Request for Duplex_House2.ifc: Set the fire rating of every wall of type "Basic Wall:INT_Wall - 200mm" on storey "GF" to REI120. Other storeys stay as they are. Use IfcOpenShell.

First a look at what the model holds.

```python
import ifcopenshell
import ifcopenshell.util.element

model = ifcopenshell.open("Duplex_House2.ifc")
print(model.schema)
storey = next(s for s in model.by_type("IfcBuildingStorey") if s.Name == "GF")
walls = [e for e in ifcopenshell.util.element.get_decomposition(storey) if e.is_a("IfcWall")]
seen = {}
for e in walls:
    element_type = ifcopenshell.util.element.get_type(e)
    key = (element_type.Name if element_type != e and element_type else None, ifcopenshell.util.element.get_pset(e, "Pset_WallCommon", "FireRating"))
    seen[key] = seen.get(key, 0) + 1
for (name, value), count in sorted(seen.items(), key=str):
    print(count, "x", name, "|", value)
```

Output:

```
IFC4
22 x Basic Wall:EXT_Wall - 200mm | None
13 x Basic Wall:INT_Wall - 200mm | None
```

```python
import ifcopenshell
import ifcopenshell.api.pset
import ifcopenshell.util.element

model = ifcopenshell.open("Duplex_House2.ifc")

storey = next(s for s in model.by_type("IfcBuildingStorey") if s.Name == "GF")
walls = [e for e in ifcopenshell.util.element.get_decomposition(storey) if e.is_a("IfcWall")]

count = 0
for e in walls:
    element_type = ifcopenshell.util.element.get_type(e)
    if element_type in (None, e) or element_type.Name != "Basic Wall:INT_Wall - 200mm":
        continue
    # add_pset returns the element's existing set when there is one.
    pset = ifcopenshell.api.pset.add_pset(model, product=e, name="Pset_WallCommon")
    ifcopenshell.api.pset.edit_pset(model, pset=pset, properties={"FireRating": "REI120"})
    count += 1

print(count, "walls updated")

model.write("Duplex_House2_rev.ifc")
```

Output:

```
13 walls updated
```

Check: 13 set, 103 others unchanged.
